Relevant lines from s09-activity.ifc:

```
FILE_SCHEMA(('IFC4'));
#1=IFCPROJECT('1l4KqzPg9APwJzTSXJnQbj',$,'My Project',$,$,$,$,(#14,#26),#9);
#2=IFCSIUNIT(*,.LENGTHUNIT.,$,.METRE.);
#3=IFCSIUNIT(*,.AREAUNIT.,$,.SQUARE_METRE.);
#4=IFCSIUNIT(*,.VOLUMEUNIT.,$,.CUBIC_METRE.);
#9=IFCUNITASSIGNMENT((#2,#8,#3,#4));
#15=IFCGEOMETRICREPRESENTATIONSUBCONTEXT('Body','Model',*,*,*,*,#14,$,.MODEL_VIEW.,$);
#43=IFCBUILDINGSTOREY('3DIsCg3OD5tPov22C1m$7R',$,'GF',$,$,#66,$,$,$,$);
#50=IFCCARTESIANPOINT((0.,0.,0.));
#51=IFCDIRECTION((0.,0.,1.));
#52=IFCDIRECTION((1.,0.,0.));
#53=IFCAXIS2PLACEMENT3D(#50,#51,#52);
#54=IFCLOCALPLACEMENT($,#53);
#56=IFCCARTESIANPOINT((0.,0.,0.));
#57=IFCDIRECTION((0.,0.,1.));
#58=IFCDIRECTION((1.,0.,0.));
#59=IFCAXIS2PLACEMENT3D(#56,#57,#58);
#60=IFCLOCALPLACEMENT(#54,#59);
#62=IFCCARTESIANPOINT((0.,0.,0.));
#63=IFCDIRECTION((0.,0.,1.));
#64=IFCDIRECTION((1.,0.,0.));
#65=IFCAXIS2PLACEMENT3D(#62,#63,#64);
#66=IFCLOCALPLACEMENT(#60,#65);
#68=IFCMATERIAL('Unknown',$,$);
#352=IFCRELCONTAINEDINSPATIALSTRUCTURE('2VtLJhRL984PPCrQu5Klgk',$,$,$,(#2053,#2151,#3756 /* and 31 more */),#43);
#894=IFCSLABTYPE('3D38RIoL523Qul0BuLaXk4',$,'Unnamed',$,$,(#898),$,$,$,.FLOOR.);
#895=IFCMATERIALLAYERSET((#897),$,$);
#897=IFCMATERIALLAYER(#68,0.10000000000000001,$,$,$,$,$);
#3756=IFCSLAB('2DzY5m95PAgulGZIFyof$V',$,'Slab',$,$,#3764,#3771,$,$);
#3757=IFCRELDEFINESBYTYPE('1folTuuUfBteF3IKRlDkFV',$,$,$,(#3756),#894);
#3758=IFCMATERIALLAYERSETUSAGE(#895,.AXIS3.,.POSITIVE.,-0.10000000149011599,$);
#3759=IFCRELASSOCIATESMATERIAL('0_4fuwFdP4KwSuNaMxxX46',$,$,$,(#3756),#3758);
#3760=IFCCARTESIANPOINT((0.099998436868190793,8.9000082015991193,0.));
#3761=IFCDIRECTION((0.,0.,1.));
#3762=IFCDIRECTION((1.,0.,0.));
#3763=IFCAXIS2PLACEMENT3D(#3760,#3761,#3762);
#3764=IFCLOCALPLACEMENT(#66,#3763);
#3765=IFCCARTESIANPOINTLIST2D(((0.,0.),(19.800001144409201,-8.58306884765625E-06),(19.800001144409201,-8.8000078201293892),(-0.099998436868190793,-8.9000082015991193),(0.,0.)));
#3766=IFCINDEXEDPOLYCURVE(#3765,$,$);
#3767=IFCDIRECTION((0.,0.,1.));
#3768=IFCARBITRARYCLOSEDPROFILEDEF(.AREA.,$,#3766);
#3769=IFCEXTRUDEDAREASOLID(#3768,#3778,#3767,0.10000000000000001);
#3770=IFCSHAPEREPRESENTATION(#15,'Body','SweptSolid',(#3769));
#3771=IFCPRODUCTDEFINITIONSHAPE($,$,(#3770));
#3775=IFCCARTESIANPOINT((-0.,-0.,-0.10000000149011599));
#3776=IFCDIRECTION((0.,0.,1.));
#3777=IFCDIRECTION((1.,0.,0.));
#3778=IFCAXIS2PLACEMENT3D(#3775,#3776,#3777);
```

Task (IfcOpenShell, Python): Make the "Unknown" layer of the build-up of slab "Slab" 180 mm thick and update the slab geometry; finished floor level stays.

```python
import ifcopenshell
import ifcopenshell.util.element
import ifcopenshell.util.representation
import ifcopenshell.util.unit

model = ifcopenshell.open("s09-activity.ifc")
unit_scale = ifcopenshell.util.unit.calculate_unit_scale(model)

layer_set = model.by_id(895)
layer = next(l for l in layer_set.MaterialLayers if l.Material and l.Material.Name == "Unknown")
change = 0.18 / unit_scale - layer.LayerThickness
layer.LayerThickness += change

# Geometry does not follow the layer set by itself.
slabs = [e for e in ifcopenshell.util.element.get_elements_by_material(model, layer_set) if e.is_a("IfcSlab")]
for slab in sorted(slabs, key=lambda e: e.id()):
    body = ifcopenshell.util.representation.get_representation(slab, "Model", "Body")
    solid = body.Items[0]
    old_depth = solid.Depth
    solid.Depth += change
    # Extruded upwards: lower the start of the extrusion so the top stays.
    x, y, z = solid.Position.Location.Coordinates
    solid.Position.Location = model.createIfcCartesianPoint((x, y, z - change))
    print(slab.id(), f"{old_depth:g} -> {solid.Depth:g}")

# The layers are counted up from the underside, which has moved.
for usage in {ifcopenshell.util.element.get_material(slab) for slab in slabs}:
    usage.OffsetFromReferenceLine -= change

model.write("s09-activity-out.ifc")
```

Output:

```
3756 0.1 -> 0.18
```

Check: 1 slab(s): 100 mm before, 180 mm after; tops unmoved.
